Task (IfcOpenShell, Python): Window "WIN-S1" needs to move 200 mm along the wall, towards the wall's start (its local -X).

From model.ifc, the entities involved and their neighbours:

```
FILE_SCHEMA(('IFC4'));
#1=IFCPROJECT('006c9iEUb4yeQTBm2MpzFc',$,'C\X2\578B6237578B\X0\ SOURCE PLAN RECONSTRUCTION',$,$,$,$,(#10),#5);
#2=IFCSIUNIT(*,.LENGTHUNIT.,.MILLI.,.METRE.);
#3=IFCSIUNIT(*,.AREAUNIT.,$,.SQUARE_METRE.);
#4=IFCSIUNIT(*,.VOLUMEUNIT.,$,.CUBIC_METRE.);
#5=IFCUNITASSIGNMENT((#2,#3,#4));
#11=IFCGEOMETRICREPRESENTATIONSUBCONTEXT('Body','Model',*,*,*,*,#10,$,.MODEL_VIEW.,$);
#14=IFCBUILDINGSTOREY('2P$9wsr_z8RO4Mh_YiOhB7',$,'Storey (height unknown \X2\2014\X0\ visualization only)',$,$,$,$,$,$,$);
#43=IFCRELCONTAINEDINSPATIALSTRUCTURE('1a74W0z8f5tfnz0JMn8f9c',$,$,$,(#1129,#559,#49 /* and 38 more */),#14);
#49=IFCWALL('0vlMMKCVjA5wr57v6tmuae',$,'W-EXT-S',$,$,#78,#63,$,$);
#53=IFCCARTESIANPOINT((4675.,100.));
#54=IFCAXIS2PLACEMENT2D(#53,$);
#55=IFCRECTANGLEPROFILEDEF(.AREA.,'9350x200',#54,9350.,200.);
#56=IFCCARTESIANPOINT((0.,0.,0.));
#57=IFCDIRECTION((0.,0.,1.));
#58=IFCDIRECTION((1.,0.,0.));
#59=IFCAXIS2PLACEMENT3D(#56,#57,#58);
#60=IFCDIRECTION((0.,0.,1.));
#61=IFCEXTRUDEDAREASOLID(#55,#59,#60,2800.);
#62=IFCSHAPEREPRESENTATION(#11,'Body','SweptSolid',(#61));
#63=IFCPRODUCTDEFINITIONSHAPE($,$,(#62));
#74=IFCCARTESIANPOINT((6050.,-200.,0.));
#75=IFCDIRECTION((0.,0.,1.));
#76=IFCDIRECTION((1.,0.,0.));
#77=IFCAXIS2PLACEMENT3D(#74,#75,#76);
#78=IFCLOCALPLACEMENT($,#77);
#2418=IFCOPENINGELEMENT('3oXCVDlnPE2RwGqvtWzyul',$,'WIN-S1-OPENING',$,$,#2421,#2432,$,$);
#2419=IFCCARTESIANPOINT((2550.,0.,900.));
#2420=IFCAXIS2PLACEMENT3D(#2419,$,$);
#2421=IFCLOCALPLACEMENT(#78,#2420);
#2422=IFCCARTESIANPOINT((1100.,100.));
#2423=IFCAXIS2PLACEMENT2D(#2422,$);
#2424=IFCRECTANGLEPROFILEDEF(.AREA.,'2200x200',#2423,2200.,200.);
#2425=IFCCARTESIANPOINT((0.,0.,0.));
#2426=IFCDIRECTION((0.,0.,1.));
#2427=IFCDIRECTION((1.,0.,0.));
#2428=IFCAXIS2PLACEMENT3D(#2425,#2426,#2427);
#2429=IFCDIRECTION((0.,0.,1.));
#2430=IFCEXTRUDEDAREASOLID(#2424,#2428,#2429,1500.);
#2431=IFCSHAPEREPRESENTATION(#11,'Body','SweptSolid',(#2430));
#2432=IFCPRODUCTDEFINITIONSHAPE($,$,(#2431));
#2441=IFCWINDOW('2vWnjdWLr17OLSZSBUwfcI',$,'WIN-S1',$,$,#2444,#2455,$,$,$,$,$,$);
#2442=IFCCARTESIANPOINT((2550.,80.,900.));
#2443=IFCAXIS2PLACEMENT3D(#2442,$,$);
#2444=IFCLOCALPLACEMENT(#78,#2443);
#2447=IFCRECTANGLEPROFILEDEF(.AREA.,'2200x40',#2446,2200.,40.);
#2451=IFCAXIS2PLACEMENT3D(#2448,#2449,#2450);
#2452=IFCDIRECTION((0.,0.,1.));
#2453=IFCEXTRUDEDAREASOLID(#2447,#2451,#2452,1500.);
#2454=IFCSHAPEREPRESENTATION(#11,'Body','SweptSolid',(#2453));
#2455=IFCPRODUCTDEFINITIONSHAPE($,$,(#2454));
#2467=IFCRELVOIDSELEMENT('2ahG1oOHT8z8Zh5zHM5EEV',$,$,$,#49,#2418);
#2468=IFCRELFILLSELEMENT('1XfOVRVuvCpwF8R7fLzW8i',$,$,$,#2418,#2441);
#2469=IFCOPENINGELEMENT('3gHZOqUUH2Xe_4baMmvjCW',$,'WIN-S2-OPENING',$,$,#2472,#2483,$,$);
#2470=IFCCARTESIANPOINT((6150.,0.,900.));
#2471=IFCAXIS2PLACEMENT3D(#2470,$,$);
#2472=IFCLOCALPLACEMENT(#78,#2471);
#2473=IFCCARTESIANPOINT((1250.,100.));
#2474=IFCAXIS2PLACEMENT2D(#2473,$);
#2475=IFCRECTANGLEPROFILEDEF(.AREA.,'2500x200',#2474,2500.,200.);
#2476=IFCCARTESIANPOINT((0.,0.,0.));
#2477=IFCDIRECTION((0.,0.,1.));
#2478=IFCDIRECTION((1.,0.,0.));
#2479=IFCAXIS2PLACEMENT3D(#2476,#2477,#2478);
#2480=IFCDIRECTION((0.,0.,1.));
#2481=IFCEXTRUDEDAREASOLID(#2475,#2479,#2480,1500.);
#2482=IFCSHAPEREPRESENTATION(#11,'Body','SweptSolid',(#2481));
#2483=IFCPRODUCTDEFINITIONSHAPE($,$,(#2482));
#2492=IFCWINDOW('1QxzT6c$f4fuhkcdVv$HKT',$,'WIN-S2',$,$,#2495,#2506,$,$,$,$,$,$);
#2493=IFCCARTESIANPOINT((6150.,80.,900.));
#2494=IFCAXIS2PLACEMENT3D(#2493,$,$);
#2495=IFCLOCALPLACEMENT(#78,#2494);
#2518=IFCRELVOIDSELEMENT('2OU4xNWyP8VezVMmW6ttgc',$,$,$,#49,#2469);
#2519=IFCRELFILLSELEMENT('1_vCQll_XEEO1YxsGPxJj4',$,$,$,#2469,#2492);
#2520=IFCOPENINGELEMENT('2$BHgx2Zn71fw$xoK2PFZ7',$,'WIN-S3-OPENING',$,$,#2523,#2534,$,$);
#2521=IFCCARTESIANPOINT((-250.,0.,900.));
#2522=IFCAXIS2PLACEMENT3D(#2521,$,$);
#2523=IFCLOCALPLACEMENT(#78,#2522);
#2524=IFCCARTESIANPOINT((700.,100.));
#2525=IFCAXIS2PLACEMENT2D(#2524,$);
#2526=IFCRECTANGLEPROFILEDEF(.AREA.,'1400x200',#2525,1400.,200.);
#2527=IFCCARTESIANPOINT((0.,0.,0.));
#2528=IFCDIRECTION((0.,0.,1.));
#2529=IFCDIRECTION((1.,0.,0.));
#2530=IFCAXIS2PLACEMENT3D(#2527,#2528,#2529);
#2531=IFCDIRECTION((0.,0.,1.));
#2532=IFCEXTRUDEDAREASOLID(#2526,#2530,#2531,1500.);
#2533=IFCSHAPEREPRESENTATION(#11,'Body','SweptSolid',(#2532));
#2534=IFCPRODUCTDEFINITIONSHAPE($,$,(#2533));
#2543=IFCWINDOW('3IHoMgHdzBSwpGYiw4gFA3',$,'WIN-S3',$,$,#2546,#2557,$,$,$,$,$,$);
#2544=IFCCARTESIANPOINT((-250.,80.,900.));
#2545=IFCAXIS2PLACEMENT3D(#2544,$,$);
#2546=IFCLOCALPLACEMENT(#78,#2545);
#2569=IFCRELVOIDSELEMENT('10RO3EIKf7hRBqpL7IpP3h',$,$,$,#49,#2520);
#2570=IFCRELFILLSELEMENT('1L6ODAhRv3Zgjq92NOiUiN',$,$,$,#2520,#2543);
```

```python
import ifcopenshell
import ifcopenshell.api.geometry
import ifcopenshell.util.placement
import ifcopenshell.util.unit

model = ifcopenshell.open("model.ifc")
unit_scale = ifcopenshell.util.unit.calculate_unit_scale(model)

window = model.by_guid("2vWnjdWLr17OLSZSBUwfcI")
opening = window.FillsVoids[0].RelatingOpeningElement
wall = opening.VoidsElements[0].RelatingBuildingElement

wall_matrix = ifcopenshell.util.placement.get_local_placement(wall.ObjectPlacement)
shift = wall_matrix[:3, 0] * -0.2 / unit_scale
before = ifcopenshell.util.placement.get_local_placement(window.ObjectPlacement)[:3, 3].copy()

# The window is not placed relative to its opening, so move both.
for product in (opening, window):
    matrix = ifcopenshell.util.placement.get_local_placement(product.ObjectPlacement)
    matrix[:3, 3] += shift
    ifcopenshell.api.geometry.edit_object_placement(model, product=product, matrix=matrix, is_si=False)

after = ifcopenshell.util.placement.get_local_placement(window.ObjectPlacement)[:3, 3]
print("window moved by", (after - before).round(3) + 0.0)

model.write("model_rev.ifc")
```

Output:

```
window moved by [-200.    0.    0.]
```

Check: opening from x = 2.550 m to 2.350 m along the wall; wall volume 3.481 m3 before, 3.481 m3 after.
